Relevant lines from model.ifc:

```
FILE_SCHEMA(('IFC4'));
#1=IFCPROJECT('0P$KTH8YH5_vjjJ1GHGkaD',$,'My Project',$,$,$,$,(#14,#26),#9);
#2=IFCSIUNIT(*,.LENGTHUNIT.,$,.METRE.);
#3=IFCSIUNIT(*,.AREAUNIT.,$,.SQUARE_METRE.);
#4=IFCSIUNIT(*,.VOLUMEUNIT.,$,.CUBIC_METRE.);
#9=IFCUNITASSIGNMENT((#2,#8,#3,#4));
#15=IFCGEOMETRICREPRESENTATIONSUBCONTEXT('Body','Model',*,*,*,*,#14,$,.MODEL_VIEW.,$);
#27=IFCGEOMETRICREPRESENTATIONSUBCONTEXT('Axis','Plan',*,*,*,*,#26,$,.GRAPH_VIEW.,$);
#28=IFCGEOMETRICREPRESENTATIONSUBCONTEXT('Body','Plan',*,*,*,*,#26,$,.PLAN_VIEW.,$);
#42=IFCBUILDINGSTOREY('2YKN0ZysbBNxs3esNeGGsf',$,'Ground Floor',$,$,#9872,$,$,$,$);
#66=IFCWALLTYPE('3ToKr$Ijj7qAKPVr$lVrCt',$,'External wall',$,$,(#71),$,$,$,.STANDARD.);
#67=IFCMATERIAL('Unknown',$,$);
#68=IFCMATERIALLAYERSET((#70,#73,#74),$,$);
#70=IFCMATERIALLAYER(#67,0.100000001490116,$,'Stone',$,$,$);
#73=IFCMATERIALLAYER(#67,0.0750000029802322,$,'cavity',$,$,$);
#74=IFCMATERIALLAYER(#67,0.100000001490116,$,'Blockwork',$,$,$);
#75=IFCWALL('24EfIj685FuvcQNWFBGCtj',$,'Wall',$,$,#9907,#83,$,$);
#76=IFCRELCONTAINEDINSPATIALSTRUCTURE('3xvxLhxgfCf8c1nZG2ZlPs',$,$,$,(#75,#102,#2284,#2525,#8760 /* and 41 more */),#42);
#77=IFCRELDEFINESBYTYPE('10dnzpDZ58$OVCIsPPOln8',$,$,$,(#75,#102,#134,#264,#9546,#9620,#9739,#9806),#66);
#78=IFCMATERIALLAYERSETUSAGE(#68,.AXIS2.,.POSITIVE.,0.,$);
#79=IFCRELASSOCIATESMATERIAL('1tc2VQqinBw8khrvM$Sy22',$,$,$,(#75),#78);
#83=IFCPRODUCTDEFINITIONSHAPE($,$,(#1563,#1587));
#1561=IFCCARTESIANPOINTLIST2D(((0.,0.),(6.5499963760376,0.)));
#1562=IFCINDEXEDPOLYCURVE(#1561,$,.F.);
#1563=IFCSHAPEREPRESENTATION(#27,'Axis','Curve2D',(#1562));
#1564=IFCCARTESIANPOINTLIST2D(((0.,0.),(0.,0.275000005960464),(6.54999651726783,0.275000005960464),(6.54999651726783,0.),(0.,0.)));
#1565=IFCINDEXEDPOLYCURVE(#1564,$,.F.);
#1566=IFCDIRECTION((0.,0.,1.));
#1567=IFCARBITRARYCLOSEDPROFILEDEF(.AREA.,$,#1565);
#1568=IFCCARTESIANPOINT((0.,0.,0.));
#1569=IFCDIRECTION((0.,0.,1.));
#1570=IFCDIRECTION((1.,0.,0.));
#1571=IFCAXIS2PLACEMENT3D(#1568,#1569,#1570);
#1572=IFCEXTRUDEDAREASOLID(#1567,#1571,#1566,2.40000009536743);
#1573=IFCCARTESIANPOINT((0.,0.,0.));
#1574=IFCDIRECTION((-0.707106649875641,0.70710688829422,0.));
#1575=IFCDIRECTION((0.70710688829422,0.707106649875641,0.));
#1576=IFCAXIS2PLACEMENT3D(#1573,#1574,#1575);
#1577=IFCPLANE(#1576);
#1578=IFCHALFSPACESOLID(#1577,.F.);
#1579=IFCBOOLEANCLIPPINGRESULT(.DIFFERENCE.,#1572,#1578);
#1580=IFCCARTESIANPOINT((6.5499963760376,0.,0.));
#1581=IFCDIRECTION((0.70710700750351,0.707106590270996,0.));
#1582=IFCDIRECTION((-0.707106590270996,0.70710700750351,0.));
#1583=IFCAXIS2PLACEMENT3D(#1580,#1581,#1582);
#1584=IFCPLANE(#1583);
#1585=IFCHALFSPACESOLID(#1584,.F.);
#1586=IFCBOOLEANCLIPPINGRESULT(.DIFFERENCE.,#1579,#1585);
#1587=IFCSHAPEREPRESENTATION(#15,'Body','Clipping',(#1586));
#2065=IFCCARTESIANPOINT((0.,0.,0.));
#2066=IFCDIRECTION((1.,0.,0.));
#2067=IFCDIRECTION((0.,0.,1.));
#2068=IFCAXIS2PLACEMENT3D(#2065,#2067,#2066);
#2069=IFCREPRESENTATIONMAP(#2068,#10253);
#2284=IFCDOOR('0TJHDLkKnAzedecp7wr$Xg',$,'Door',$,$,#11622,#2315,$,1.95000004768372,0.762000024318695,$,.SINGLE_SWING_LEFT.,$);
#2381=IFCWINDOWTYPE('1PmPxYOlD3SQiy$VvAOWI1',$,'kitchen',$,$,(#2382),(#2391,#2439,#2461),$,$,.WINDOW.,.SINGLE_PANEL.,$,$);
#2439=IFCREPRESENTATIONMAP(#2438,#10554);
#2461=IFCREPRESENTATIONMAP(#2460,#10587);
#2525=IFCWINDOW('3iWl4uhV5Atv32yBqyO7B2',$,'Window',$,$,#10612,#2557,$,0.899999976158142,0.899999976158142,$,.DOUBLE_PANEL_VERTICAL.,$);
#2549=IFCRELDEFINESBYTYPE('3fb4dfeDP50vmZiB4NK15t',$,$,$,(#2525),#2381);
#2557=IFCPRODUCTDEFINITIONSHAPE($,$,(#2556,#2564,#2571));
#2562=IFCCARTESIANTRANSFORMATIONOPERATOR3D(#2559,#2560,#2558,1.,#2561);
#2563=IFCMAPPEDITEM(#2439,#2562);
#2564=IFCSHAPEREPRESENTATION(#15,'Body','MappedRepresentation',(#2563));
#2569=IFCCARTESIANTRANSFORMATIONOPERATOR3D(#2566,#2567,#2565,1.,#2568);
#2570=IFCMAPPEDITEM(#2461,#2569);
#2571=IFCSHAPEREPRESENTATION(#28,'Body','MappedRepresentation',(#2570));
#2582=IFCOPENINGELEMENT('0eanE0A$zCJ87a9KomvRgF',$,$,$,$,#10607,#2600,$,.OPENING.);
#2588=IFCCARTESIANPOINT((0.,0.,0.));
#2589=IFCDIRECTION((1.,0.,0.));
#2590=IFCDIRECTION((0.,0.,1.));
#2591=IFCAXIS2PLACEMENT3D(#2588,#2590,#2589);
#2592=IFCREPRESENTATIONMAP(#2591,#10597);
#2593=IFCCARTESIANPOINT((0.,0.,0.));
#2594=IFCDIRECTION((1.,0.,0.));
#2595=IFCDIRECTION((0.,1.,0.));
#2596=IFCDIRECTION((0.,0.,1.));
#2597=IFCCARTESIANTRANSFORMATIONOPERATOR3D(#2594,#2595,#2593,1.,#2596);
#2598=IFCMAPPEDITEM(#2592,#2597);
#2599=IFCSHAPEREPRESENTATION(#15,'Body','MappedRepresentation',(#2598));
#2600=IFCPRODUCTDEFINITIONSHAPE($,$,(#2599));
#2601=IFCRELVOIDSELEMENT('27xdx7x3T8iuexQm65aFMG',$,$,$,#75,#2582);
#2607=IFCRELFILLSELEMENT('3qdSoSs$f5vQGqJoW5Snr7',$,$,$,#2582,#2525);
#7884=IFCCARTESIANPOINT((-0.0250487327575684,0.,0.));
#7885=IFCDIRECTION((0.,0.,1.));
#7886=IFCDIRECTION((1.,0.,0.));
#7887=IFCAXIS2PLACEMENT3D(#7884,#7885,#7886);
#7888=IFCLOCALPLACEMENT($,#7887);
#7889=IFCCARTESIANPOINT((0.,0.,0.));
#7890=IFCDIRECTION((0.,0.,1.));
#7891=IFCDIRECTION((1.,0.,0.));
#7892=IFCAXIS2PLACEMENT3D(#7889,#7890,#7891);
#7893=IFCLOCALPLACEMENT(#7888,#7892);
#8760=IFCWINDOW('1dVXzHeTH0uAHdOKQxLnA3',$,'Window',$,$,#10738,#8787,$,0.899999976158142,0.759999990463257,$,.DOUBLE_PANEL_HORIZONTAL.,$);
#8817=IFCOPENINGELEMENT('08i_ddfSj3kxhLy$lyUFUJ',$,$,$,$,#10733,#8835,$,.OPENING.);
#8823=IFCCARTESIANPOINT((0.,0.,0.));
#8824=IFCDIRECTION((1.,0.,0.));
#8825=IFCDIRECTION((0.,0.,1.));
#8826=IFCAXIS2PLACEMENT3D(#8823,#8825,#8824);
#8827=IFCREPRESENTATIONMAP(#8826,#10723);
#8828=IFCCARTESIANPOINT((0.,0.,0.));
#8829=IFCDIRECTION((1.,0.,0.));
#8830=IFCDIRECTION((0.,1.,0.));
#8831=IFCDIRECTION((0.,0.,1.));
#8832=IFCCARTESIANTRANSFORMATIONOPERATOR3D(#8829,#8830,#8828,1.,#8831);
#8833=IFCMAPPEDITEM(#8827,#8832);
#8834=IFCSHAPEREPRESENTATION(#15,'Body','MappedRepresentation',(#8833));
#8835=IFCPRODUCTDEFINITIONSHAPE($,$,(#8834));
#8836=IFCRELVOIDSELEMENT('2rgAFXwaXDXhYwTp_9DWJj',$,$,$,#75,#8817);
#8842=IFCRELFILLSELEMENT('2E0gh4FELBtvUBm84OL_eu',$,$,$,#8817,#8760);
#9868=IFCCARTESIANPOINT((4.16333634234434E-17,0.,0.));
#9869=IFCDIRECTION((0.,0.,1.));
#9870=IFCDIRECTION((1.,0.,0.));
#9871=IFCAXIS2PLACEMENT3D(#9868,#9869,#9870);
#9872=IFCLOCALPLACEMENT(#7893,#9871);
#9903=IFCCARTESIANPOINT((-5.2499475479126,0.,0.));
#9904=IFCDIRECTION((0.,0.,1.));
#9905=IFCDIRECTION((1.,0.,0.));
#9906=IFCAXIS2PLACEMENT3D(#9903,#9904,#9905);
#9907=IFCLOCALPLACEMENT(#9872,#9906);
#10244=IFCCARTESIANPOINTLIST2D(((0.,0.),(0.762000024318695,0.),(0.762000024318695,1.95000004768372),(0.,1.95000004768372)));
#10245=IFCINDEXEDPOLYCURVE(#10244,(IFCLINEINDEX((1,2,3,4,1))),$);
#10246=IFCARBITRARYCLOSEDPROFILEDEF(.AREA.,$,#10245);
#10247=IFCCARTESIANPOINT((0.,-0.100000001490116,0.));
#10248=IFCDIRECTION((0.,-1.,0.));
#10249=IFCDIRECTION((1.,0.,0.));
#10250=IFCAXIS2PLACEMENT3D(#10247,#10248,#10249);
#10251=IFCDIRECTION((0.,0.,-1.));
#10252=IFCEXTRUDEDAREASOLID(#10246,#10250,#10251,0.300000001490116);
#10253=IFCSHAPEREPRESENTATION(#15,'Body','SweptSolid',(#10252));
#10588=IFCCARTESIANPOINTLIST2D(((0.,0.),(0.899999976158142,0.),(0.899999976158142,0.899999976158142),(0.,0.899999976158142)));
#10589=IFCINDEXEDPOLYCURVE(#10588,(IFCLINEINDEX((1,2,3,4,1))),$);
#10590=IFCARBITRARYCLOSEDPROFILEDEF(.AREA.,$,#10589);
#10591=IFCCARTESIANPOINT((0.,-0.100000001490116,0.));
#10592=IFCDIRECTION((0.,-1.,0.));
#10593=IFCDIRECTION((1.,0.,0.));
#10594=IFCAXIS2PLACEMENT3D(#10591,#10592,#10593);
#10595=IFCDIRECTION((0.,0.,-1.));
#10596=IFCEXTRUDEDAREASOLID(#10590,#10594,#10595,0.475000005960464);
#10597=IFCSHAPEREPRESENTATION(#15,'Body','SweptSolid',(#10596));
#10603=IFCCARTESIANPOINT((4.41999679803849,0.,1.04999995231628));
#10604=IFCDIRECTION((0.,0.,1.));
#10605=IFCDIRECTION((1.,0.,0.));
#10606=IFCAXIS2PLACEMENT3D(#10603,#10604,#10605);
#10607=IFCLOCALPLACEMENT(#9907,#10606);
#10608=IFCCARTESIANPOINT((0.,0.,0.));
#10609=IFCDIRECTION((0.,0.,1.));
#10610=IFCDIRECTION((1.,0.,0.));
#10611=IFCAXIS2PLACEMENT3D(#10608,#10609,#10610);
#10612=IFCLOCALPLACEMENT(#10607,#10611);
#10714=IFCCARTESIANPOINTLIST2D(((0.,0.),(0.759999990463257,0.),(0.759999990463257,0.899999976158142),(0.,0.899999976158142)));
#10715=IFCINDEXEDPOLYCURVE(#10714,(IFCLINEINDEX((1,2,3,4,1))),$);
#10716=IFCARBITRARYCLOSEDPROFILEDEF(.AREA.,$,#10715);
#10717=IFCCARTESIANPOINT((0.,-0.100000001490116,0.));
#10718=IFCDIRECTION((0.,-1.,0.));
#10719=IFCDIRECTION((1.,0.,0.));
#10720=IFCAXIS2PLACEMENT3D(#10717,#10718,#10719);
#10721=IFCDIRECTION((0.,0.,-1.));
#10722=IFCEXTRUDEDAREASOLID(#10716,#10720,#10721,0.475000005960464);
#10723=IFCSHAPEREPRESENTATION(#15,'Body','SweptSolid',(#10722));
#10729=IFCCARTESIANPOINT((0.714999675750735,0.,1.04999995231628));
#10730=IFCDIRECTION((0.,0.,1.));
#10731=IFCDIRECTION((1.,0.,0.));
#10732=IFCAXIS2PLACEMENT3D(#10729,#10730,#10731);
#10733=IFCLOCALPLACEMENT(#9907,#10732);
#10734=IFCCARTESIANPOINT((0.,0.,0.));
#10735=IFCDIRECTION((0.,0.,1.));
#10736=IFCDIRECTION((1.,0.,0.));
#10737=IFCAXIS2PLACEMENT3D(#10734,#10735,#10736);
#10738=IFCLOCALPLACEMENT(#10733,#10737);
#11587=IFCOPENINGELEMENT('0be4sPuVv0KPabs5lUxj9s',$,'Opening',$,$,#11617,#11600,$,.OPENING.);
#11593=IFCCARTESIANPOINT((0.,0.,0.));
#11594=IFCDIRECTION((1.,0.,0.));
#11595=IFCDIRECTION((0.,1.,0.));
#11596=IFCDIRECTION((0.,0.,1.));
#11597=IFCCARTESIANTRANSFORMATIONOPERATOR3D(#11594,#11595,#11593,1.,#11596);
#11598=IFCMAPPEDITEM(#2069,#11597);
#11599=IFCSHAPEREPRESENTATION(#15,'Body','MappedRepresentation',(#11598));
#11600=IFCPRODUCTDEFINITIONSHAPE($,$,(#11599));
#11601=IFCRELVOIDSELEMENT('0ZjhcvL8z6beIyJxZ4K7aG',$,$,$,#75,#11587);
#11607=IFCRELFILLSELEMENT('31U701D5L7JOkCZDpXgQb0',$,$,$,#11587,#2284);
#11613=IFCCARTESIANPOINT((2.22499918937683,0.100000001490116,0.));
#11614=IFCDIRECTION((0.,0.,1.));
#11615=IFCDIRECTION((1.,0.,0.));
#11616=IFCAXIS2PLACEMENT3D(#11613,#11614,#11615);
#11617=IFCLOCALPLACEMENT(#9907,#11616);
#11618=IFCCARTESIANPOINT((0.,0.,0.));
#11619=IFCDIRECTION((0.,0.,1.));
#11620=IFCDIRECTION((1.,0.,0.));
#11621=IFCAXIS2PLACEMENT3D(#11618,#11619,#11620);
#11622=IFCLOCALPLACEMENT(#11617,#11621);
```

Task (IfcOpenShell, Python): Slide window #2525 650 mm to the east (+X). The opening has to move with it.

```python
import ifcopenshell
import ifcopenshell.api.geometry
import ifcopenshell.util.placement
import ifcopenshell.util.unit

model = ifcopenshell.open("model.ifc")
unit_scale = ifcopenshell.util.unit.calculate_unit_scale(model)

window = model.by_id(2525)
opening = window.FillsVoids[0].RelatingOpeningElement
wall = opening.VoidsElements[0].RelatingBuildingElement

wall_matrix = ifcopenshell.util.placement.get_local_placement(wall.ObjectPlacement)
shift = wall_matrix[:3, 0] * 0.65 / unit_scale
before = ifcopenshell.util.placement.get_local_placement(window.ObjectPlacement)[:3, 3].copy()

# The window is placed relative to its opening, so it follows when the opening moves.
matrix = ifcopenshell.util.placement.get_local_placement(opening.ObjectPlacement)
matrix[:3, 3] += shift
ifcopenshell.api.geometry.edit_object_placement(
    model, product=opening, matrix=matrix, is_si=False, should_transform_children=True
)

after = ifcopenshell.util.placement.get_local_placement(window.ObjectPlacement)[:3, 3]
print("window moved by", (after - before).round(3) + 0.0)

model.write("model_v2.ifc")
```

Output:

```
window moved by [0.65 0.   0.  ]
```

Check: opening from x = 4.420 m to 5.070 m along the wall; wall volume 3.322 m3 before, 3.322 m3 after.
